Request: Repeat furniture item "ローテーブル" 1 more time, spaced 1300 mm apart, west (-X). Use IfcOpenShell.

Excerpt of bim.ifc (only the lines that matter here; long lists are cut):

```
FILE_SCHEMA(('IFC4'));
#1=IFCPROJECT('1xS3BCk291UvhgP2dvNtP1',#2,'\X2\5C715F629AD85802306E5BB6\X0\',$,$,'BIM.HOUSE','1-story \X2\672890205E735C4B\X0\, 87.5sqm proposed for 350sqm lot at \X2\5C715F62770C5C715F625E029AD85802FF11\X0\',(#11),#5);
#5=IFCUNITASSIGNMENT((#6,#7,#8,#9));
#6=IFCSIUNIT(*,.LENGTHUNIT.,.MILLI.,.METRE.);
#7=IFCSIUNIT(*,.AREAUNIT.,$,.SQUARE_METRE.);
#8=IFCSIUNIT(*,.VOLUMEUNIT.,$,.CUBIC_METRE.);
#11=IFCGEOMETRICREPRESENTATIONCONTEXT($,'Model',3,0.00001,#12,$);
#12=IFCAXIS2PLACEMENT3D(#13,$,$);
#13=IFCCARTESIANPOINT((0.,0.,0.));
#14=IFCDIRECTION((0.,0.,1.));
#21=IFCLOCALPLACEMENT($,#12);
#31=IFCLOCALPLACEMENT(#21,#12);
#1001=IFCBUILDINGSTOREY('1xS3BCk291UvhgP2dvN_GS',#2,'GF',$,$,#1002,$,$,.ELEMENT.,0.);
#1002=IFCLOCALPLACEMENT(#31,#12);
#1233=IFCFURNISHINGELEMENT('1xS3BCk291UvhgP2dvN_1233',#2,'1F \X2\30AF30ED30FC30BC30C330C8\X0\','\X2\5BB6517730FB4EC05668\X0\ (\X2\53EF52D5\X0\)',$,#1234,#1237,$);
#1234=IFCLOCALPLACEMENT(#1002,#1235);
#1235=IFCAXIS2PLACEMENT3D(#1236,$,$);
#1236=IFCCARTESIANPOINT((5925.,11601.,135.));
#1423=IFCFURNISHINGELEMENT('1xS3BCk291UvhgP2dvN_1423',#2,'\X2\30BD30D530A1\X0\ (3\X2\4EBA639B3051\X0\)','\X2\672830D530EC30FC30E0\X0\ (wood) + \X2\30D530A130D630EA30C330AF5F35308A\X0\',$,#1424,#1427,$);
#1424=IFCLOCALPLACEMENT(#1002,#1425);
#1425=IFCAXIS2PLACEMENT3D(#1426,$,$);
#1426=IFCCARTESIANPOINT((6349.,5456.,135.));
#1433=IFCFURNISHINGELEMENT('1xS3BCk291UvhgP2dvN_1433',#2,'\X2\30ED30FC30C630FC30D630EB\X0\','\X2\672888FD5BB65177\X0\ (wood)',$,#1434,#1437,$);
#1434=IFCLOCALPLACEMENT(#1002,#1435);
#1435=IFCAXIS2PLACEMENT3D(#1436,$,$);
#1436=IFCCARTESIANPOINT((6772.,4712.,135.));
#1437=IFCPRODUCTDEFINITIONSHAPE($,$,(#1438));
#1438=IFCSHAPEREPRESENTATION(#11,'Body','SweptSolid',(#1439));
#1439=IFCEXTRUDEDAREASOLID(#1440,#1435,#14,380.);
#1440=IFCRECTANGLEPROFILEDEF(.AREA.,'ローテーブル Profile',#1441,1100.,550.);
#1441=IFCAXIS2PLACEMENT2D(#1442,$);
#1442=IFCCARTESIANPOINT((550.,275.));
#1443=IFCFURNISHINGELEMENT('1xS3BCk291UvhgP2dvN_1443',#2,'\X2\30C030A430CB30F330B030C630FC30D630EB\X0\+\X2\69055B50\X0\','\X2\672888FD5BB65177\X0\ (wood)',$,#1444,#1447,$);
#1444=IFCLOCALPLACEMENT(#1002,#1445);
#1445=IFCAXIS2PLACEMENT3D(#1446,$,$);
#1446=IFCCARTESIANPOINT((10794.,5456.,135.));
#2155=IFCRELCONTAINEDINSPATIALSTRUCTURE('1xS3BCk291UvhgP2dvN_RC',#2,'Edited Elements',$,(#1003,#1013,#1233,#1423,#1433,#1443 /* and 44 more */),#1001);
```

```python
import numpy as np
import ifcopenshell
import ifcopenshell.api.geometry
import ifcopenshell.api.root
import ifcopenshell.util.element
import ifcopenshell.util.placement
import ifcopenshell.util.unit

model = ifcopenshell.open("bim.ifc")
unit_scale = ifcopenshell.util.unit.calculate_unit_scale(model)


def reuse_history(source, copy):
    """copy_class also copies each property set's owner history, people and application; keep the originals."""
    for rel in copy.IsDefinedBy:
        if rel.is_a("IfcRelDefinesByProperties") and (history := rel.RelatingPropertyDefinition.OwnerHistory):
            rel.RelatingPropertyDefinition.OwnerHistory = source.OwnerHistory
            ifcopenshell.util.element.remove_deep2(model, history)


source = model.by_guid("1xS3BCk291UvhgP2dvN_1433")
base = ifcopenshell.util.placement.get_local_placement(source.ObjectPlacement)
step = np.array([-1.0, 0.0, 0.0]) * 1.3 / unit_scale

for i in range(1, 2):
    copy = ifcopenshell.api.root.copy_class(model, product=source)
    copy.Representation = ifcopenshell.util.element.copy_deep(
        model, source.Representation, exclude=["IfcGeometricRepresentationContext", "IfcRepresentationMap"]
    )
    reuse_history(source, copy)
    matrix = base.copy()
    matrix[:3, 3] += i * step
    print("added at", matrix[:3, 3].round(3) + 0.0)
    ifcopenshell.api.geometry.edit_object_placement(model, product=copy, matrix=matrix, is_si=False)

model.write("bim_edited.ifc")
```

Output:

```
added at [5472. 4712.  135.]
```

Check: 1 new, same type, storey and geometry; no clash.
